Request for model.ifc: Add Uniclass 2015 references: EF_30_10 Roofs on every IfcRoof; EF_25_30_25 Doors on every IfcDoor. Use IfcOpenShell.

First a look at what the model holds.

```python
import ifcopenshell

model = ifcopenshell.open("model.ifc")
print(model.schema)
print("classifications:", [c.Name for c in model.by_type("IfcClassification")])
for ifc_class in ("IfcDoor", "IfcRoof", "IfcStair", "IfcWall", "IfcWindow"):
    print(ifc_class, len(model.by_type(ifc_class)))
```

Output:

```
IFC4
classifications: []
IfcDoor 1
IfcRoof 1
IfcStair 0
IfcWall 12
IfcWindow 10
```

```python
import ifcopenshell
import ifcopenshell.api.classification

model = ifcopenshell.open("model.ifc")

system = ifcopenshell.api.classification.add_classification(model, classification="Uniclass 2015")

codes = {
    "IfcRoof": ("EF_30_10", "Roofs"),
    "IfcDoor": ("EF_25_30_25", "Doors"),
}
for ifc_class, (code, name) in codes.items():
    products = model.by_type(ifc_class)
    ifcopenshell.api.classification.add_reference(
        model, products=products, classification=system, identification=code, name=name
    )
    print(code, len(products))

model.write("model_rev.ifc")
```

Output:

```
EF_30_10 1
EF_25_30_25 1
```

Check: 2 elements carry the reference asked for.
